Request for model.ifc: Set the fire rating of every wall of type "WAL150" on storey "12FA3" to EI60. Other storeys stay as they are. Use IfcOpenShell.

First a look at what the model holds.

```python
import ifcopenshell
import ifcopenshell.util.element

model = ifcopenshell.open("model.ifc")
print(model.schema)
storey = next(s for s in model.by_type("IfcBuildingStorey") if s.Name == "12FA3")
walls = [e for e in ifcopenshell.util.element.get_decomposition(storey) if e.is_a("IfcWall")]
seen = {}
for e in walls:
    element_type = ifcopenshell.util.element.get_type(e)
    key = (element_type.Name if element_type != e and element_type else None, ifcopenshell.util.element.get_pset(e, "Pset_WallCommon", "FireRating"))
    seen[key] = seen.get(key, 0) + 1
for (name, value), count in sorted(seen.items(), key=str):
    print(count, "x", name, "|", value)
```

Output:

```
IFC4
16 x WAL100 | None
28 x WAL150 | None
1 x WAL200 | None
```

```python
import ifcopenshell
import ifcopenshell.api.pset
import ifcopenshell.util.element

model = ifcopenshell.open("model.ifc")

storey = next(s for s in model.by_type("IfcBuildingStorey") if s.Name == "12FA3")
walls = [e for e in ifcopenshell.util.element.get_decomposition(storey) if e.is_a("IfcWall")]

count = 0
for e in walls:
    element_type = ifcopenshell.util.element.get_type(e)
    if element_type in (None, e) or element_type.Name != "WAL150":
        continue
    # add_pset returns the element's existing set when there is one.
    pset = ifcopenshell.api.pset.add_pset(model, product=e, name="Pset_WallCommon")
    ifcopenshell.api.pset.edit_pset(model, pset=pset, properties={"FireRating": "EI60"})
    count += 1

print(count, "walls updated")

model.write("model_updated.ifc")
```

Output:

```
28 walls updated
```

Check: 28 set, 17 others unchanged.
